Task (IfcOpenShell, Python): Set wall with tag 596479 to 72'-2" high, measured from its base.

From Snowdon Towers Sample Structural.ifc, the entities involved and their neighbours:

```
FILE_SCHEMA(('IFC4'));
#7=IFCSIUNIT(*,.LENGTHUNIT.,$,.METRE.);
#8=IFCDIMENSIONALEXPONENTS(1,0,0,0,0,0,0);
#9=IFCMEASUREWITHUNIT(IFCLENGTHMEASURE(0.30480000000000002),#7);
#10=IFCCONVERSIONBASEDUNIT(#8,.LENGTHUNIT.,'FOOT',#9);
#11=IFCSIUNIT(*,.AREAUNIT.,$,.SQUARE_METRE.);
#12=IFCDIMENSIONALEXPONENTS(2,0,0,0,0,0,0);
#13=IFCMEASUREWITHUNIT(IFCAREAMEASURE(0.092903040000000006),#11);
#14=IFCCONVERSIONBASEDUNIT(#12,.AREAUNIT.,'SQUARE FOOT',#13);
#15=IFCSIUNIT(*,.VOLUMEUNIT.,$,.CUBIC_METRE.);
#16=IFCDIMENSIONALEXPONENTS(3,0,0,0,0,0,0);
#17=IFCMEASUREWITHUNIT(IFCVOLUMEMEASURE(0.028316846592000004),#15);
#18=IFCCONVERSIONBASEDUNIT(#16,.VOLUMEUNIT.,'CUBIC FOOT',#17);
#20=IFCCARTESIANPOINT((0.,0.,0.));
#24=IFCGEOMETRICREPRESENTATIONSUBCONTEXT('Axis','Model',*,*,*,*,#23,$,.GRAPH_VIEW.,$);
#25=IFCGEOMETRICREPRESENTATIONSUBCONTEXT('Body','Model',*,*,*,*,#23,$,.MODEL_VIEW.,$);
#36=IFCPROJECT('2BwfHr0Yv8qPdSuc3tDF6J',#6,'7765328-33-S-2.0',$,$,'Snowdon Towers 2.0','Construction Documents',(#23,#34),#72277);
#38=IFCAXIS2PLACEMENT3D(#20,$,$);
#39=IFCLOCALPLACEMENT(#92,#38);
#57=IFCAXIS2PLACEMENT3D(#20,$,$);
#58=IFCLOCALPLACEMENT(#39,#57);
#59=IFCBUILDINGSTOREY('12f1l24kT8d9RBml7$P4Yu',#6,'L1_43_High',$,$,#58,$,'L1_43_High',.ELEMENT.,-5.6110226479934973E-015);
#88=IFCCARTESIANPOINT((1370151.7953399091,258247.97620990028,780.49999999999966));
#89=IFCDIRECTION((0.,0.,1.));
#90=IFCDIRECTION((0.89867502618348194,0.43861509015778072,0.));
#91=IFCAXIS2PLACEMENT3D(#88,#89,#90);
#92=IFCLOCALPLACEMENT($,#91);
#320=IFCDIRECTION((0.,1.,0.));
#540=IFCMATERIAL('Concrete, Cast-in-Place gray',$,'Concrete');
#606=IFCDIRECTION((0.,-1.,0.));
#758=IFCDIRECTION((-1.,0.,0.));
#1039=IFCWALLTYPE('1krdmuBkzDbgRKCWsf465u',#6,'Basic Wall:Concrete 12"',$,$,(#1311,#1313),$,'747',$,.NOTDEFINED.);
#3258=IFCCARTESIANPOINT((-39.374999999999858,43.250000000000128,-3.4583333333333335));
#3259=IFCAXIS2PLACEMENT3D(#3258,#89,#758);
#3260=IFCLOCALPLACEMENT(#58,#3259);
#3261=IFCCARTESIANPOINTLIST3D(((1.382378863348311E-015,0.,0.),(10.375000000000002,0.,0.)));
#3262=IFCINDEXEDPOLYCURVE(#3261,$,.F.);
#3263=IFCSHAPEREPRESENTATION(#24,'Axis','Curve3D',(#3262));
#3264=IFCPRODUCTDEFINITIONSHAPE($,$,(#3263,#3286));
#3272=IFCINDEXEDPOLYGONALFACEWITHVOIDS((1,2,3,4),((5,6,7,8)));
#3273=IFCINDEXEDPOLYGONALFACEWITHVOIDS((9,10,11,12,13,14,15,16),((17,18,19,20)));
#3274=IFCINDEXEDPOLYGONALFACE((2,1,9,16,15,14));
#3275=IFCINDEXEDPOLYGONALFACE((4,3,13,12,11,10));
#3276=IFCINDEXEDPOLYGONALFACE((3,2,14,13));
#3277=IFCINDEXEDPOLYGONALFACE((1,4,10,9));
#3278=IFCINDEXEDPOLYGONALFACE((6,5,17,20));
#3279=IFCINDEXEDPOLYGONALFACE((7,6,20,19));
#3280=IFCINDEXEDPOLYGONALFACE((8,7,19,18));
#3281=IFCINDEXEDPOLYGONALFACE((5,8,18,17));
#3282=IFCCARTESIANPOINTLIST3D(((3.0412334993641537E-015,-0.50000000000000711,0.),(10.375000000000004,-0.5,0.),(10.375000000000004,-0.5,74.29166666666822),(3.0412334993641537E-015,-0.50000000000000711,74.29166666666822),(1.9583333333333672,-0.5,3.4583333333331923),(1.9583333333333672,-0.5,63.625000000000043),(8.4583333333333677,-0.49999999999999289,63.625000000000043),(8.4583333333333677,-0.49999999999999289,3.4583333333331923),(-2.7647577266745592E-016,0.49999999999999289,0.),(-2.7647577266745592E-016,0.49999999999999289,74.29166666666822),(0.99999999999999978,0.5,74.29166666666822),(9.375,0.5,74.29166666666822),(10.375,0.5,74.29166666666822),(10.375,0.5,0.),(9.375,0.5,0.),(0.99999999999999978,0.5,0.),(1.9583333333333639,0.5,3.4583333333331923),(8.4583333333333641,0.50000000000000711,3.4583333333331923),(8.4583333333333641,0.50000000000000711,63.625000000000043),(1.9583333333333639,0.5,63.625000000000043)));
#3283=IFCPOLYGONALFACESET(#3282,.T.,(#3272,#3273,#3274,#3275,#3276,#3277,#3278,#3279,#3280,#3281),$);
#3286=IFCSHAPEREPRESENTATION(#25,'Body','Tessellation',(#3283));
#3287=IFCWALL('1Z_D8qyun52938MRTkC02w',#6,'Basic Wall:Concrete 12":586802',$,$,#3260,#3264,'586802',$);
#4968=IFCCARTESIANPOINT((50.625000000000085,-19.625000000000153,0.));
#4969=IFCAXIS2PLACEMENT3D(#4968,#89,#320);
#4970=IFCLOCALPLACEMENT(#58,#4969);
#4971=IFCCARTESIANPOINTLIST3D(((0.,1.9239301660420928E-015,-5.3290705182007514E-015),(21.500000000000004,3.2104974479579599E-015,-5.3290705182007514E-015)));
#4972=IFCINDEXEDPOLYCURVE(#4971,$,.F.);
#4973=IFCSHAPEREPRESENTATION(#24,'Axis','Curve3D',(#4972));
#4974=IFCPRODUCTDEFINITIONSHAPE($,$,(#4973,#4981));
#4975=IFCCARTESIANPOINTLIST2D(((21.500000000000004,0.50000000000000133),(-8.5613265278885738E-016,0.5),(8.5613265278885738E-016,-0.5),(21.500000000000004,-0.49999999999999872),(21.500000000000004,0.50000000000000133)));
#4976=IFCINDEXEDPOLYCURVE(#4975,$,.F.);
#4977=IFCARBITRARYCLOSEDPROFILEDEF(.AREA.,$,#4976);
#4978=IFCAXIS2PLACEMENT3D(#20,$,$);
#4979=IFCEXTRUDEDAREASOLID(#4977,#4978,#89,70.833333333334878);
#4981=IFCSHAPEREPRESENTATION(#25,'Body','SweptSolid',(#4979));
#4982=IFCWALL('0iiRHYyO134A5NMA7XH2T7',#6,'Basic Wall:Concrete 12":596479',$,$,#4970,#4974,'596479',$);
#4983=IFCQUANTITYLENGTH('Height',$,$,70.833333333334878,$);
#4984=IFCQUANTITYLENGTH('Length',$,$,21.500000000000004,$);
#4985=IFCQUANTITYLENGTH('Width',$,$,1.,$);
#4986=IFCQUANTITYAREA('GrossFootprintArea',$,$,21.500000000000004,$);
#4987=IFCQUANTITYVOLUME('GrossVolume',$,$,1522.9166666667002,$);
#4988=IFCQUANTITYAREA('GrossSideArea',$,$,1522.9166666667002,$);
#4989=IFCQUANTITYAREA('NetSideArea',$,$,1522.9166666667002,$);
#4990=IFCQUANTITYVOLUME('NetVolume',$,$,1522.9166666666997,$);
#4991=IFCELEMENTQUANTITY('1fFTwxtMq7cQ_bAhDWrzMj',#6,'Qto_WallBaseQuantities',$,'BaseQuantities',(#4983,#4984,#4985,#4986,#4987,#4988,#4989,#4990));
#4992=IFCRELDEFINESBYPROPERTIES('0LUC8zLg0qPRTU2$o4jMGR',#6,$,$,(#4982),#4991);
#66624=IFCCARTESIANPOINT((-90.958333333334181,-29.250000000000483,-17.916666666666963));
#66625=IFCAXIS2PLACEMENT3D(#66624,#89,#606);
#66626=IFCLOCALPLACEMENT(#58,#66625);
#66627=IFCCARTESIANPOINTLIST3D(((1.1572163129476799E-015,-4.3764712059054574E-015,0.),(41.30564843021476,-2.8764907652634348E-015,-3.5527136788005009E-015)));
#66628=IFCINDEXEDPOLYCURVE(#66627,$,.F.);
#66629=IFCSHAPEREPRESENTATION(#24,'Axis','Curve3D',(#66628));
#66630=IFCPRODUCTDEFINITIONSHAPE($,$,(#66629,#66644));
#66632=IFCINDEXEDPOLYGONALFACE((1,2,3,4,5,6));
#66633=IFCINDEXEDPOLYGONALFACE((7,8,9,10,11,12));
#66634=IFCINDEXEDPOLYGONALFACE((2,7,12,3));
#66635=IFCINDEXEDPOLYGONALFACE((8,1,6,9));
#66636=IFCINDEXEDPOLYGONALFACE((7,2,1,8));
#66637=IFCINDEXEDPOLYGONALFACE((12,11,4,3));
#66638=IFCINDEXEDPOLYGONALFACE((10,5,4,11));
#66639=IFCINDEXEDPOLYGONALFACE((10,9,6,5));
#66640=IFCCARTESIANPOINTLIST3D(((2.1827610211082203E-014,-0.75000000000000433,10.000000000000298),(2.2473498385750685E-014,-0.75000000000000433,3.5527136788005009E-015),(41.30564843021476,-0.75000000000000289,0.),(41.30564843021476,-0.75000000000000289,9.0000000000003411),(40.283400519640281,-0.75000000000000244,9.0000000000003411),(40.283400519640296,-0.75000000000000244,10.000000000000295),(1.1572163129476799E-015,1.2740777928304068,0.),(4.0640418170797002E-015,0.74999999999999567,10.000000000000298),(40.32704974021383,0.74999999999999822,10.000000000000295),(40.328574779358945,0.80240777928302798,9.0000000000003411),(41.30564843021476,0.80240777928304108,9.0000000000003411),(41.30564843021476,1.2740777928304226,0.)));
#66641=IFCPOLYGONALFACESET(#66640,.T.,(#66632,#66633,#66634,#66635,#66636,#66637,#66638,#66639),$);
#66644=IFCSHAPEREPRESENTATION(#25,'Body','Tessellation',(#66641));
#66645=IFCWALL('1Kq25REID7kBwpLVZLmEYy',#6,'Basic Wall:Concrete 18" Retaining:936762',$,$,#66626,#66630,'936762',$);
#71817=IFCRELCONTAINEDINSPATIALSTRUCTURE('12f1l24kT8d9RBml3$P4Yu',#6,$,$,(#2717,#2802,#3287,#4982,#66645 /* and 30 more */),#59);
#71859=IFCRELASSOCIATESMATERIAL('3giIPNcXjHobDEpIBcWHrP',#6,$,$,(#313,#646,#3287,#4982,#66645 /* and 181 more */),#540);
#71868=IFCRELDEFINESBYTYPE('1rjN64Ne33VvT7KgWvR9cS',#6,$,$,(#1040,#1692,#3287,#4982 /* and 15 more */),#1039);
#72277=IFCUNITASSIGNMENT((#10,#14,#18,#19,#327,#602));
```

```python
import ifcopenshell
import ifcopenshell.api.pset
import ifcopenshell.geom
import ifcopenshell.util.element
import ifcopenshell.util.representation
import ifcopenshell.util.shape
import ifcopenshell.util.unit

model = ifcopenshell.open("Snowdon Towers Sample Structural.ifc")
unit_scale = ifcopenshell.util.unit.calculate_unit_scale(model)
area_scale = ifcopenshell.util.unit.calculate_unit_scale(model, "AREAUNIT")
volume_scale = ifcopenshell.util.unit.calculate_unit_scale(model, "VOLUMEUNIT")
settings = ifcopenshell.geom.settings()


def volume(element):
    """Net volume in cubic metres, openings subtracted."""
    shape = ifcopenshell.geom.create_shape(settings, element)
    return ifcopenshell.util.shape.get_volume(shape.geometry)


wall = model.by_guid("0iiRHYyO134A5NMA7XH2T7")
before = volume(wall)

body = ifcopenshell.util.representation.get_representation(wall, "Model", "Body")
solid = body.Items[0]
old_height = solid.Depth
solid.Depth = 866 * 0.0254 / unit_scale
after = volume(wall)
thickness = 0.3048  # wall thickness in metres

# Update the stored height, areas and volumes.
qto = model.by_id(ifcopenshell.util.element.get_pset(wall, "Qto_WallBaseQuantities", should_inherit=False)["id"])
ifcopenshell.api.pset.edit_qto(model, qto=qto, properties={
    "Height": solid.Depth,
    "GrossVolume": ifcopenshell.util.element.get_pset(wall, "Qto_WallBaseQuantities", "GrossVolume") * solid.Depth / old_height,
    "GrossSideArea": ifcopenshell.util.element.get_pset(wall, "Qto_WallBaseQuantities", "GrossSideArea") * solid.Depth / old_height,
    "NetSideArea": after / thickness / area_scale,
    "NetVolume": after / volume_scale,
})

print(f"height {old_height:g} -> {solid.Depth:g}, volume {before:.3f} -> {after:.3f} m3")

model.write("Snowdon Towers Sample Structural-out.ifc")
```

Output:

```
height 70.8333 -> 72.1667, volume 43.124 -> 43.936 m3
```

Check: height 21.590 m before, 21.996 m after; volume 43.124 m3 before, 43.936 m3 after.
